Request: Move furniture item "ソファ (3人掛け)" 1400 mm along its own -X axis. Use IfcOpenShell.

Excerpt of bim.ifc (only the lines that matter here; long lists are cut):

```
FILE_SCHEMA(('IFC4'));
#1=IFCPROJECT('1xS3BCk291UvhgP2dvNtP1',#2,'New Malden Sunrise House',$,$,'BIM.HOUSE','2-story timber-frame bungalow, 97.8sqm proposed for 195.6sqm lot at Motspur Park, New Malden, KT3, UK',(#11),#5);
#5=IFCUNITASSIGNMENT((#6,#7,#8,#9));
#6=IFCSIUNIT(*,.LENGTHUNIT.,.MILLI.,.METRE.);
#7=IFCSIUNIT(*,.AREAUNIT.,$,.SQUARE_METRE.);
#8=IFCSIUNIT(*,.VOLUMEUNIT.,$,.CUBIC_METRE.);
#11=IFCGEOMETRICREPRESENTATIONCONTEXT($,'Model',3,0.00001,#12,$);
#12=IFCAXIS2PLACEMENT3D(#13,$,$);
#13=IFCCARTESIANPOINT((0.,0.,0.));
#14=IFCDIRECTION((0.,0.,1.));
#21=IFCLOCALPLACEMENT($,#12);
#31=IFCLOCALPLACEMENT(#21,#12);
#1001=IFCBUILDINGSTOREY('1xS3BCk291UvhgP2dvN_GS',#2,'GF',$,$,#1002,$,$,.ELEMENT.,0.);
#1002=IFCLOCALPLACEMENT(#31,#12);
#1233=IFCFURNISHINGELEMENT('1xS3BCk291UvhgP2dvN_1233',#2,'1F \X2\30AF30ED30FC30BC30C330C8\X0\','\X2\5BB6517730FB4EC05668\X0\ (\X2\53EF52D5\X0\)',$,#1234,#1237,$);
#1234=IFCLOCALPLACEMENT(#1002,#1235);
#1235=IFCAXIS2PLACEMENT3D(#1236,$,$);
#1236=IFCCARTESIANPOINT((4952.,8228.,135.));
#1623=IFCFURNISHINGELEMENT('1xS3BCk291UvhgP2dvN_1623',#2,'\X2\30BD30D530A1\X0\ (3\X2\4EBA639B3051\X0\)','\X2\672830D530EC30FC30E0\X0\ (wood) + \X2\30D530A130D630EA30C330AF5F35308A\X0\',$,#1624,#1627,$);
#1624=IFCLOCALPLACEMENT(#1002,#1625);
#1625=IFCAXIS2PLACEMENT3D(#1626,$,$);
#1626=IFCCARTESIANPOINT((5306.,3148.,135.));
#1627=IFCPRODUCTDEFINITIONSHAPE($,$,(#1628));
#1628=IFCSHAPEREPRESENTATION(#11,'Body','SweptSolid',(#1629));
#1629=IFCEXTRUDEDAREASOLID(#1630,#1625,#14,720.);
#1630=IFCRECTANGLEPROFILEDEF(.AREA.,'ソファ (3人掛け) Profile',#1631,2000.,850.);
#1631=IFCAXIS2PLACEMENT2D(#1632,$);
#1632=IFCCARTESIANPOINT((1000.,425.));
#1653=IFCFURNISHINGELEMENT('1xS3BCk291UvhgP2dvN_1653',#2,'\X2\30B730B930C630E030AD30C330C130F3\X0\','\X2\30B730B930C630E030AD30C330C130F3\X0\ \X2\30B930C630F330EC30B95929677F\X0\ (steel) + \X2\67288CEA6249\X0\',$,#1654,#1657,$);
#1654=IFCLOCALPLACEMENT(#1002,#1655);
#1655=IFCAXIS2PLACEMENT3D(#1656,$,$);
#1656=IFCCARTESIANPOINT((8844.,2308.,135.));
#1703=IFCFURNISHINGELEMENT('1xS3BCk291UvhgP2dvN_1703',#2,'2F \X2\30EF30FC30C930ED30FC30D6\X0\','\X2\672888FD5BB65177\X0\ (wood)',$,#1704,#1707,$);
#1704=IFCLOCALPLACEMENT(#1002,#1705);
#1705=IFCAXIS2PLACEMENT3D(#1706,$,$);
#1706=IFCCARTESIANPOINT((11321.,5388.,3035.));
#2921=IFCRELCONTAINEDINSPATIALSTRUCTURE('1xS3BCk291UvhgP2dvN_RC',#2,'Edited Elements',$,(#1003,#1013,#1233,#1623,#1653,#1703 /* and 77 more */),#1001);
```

```python
import ifcopenshell
import ifcopenshell.api.geometry
import ifcopenshell.util.placement

model = ifcopenshell.open("bim.ifc")

item = model.by_guid("1xS3BCk291UvhgP2dvN_1623")
matrix = ifcopenshell.util.placement.get_local_placement(item.ObjectPlacement)
matrix[:3, 3] -= matrix[:3, 0] * 1400.0
ifcopenshell.api.geometry.edit_object_placement(model, product=item, matrix=matrix, is_si=False)

print(ifcopenshell.util.placement.get_local_placement(item.ObjectPlacement).round(3) + 0.0)

model.write("bim_rev.ifc")
```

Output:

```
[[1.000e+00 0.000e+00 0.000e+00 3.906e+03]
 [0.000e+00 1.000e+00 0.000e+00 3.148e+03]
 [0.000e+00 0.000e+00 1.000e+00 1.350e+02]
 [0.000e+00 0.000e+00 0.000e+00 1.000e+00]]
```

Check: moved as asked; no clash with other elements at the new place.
